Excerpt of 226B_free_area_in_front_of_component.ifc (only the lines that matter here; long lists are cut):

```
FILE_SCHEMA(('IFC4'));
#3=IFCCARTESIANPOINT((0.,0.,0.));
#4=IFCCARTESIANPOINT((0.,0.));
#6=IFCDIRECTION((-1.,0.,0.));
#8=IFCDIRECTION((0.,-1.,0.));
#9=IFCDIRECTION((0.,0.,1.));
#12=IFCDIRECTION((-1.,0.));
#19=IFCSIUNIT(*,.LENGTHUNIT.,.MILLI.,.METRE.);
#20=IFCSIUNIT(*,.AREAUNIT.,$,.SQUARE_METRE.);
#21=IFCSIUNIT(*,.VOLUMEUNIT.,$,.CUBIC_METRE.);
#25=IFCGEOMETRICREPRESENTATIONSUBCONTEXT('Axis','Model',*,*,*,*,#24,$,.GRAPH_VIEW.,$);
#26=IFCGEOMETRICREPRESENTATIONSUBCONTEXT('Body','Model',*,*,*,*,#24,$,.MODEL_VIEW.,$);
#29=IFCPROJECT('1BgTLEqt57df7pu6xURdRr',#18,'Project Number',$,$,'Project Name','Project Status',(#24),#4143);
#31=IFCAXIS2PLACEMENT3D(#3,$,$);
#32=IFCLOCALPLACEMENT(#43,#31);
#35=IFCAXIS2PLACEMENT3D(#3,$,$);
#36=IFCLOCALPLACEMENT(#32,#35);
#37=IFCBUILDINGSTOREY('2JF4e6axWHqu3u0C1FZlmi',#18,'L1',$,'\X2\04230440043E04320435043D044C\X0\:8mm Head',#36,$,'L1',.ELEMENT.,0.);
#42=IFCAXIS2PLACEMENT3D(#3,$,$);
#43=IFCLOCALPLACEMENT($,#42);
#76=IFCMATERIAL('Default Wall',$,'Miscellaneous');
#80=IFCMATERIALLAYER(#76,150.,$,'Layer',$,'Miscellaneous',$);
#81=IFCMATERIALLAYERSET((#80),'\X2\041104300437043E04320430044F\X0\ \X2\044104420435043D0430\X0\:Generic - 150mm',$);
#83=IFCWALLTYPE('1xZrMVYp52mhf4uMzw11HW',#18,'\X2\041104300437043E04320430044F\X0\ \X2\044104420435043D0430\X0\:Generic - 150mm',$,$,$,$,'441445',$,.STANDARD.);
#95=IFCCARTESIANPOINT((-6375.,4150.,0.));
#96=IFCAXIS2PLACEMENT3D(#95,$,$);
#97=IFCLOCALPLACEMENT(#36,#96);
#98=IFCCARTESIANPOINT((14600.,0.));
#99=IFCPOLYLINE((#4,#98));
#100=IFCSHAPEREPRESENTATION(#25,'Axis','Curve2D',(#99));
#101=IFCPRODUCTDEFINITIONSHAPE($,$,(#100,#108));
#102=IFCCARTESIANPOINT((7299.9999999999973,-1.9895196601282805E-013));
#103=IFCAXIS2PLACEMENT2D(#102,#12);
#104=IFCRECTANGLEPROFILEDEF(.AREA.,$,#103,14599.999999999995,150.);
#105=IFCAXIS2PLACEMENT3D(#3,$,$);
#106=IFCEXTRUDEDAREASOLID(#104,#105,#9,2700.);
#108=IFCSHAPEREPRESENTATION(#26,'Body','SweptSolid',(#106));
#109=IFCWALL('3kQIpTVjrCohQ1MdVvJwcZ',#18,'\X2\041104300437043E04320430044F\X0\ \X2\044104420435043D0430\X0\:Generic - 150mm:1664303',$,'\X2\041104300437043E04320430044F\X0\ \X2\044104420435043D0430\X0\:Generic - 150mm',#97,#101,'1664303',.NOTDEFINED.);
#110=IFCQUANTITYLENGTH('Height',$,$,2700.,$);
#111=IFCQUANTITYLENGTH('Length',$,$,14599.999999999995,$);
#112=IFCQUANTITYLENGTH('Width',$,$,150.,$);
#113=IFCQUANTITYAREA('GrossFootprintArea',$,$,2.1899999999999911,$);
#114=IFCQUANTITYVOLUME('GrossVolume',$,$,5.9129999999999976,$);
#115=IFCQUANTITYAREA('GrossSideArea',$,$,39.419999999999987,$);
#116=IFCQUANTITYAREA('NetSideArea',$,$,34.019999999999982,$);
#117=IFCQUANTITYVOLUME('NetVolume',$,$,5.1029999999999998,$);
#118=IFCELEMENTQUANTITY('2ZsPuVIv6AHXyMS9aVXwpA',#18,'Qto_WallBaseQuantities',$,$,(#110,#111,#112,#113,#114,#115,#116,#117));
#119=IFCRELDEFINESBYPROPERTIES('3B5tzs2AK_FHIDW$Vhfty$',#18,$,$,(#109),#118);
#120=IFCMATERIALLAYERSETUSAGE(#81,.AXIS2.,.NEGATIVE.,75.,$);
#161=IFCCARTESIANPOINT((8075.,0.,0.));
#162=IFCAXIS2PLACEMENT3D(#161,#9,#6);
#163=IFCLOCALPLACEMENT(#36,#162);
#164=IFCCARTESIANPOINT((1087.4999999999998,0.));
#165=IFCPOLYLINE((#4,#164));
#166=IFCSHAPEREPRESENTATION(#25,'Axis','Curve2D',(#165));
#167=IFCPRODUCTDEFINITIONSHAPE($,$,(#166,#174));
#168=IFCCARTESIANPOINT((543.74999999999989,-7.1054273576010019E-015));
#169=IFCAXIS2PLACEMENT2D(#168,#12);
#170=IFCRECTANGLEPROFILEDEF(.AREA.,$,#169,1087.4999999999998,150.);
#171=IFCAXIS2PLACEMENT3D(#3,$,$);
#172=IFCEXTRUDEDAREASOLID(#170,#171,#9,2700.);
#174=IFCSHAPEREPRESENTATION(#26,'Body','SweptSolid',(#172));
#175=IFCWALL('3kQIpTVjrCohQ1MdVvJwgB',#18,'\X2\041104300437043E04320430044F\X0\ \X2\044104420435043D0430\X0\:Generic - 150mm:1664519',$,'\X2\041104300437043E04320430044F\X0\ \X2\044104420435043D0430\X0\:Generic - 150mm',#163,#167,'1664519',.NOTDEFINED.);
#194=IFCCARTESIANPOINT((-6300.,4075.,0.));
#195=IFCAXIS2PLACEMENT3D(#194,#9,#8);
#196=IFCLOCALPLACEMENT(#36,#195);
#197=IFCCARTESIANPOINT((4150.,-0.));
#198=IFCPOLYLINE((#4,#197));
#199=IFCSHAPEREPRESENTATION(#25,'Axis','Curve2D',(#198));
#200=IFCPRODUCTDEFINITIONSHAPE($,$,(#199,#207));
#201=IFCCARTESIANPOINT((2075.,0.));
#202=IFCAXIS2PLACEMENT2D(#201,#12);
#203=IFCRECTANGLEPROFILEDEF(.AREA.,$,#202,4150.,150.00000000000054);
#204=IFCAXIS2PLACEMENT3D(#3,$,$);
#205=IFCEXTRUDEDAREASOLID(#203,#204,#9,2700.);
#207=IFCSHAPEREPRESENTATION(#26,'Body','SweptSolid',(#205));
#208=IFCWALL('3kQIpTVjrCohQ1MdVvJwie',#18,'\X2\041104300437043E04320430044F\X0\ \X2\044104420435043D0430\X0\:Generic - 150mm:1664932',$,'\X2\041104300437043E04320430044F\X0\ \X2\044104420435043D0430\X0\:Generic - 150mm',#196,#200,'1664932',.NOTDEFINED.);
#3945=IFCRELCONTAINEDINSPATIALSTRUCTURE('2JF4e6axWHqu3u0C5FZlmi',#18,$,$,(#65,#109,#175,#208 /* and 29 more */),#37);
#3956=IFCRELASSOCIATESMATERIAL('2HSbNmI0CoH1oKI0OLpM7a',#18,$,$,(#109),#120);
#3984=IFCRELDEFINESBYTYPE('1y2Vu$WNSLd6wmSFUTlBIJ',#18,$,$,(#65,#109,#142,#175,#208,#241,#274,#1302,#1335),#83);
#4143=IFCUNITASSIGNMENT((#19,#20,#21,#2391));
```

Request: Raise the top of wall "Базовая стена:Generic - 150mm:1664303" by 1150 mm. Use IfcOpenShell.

```python
import ifcopenshell
import ifcopenshell.api.pset
import ifcopenshell.geom
import ifcopenshell.util.element
import ifcopenshell.util.representation
import ifcopenshell.util.shape
import ifcopenshell.util.unit

model = ifcopenshell.open("226B_free_area_in_front_of_component.ifc")
unit_scale = ifcopenshell.util.unit.calculate_unit_scale(model)
area_scale = ifcopenshell.util.unit.calculate_unit_scale(model, "AREAUNIT")
volume_scale = ifcopenshell.util.unit.calculate_unit_scale(model, "VOLUMEUNIT")
settings = ifcopenshell.geom.settings()


def volume(element):
    """Net volume in cubic metres, openings subtracted."""
    shape = ifcopenshell.geom.create_shape(settings, element)
    return ifcopenshell.util.shape.get_volume(shape.geometry)


wall = model.by_guid("3kQIpTVjrCohQ1MdVvJwcZ")
before = volume(wall)

body = ifcopenshell.util.representation.get_representation(wall, "Model", "Body")
solid = body.Items[0]
old_height = solid.Depth
solid.Depth += 1.15 / unit_scale
after = volume(wall)
thickness = 0.15  # wall thickness in metres

# Update the stored height, areas and volumes.
qto = model.by_id(ifcopenshell.util.element.get_pset(wall, "Qto_WallBaseQuantities", should_inherit=False)["id"])
ifcopenshell.api.pset.edit_qto(model, qto=qto, properties={
    "Height": solid.Depth,
    "GrossVolume": ifcopenshell.util.element.get_pset(wall, "Qto_WallBaseQuantities", "GrossVolume") * solid.Depth / old_height,
    "GrossSideArea": ifcopenshell.util.element.get_pset(wall, "Qto_WallBaseQuantities", "GrossSideArea") * solid.Depth / old_height,
    "NetSideArea": after / thickness / area_scale,
    "NetVolume": after / volume_scale,
})

print(f"height {old_height:g} -> {solid.Depth:g}, volume {before:.3f} -> {after:.3f} m3")

model.write("226B_free_area_in_front_of_component_edited.ifc")
```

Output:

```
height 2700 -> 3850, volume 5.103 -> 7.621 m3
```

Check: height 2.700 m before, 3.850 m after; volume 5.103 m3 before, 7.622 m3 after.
